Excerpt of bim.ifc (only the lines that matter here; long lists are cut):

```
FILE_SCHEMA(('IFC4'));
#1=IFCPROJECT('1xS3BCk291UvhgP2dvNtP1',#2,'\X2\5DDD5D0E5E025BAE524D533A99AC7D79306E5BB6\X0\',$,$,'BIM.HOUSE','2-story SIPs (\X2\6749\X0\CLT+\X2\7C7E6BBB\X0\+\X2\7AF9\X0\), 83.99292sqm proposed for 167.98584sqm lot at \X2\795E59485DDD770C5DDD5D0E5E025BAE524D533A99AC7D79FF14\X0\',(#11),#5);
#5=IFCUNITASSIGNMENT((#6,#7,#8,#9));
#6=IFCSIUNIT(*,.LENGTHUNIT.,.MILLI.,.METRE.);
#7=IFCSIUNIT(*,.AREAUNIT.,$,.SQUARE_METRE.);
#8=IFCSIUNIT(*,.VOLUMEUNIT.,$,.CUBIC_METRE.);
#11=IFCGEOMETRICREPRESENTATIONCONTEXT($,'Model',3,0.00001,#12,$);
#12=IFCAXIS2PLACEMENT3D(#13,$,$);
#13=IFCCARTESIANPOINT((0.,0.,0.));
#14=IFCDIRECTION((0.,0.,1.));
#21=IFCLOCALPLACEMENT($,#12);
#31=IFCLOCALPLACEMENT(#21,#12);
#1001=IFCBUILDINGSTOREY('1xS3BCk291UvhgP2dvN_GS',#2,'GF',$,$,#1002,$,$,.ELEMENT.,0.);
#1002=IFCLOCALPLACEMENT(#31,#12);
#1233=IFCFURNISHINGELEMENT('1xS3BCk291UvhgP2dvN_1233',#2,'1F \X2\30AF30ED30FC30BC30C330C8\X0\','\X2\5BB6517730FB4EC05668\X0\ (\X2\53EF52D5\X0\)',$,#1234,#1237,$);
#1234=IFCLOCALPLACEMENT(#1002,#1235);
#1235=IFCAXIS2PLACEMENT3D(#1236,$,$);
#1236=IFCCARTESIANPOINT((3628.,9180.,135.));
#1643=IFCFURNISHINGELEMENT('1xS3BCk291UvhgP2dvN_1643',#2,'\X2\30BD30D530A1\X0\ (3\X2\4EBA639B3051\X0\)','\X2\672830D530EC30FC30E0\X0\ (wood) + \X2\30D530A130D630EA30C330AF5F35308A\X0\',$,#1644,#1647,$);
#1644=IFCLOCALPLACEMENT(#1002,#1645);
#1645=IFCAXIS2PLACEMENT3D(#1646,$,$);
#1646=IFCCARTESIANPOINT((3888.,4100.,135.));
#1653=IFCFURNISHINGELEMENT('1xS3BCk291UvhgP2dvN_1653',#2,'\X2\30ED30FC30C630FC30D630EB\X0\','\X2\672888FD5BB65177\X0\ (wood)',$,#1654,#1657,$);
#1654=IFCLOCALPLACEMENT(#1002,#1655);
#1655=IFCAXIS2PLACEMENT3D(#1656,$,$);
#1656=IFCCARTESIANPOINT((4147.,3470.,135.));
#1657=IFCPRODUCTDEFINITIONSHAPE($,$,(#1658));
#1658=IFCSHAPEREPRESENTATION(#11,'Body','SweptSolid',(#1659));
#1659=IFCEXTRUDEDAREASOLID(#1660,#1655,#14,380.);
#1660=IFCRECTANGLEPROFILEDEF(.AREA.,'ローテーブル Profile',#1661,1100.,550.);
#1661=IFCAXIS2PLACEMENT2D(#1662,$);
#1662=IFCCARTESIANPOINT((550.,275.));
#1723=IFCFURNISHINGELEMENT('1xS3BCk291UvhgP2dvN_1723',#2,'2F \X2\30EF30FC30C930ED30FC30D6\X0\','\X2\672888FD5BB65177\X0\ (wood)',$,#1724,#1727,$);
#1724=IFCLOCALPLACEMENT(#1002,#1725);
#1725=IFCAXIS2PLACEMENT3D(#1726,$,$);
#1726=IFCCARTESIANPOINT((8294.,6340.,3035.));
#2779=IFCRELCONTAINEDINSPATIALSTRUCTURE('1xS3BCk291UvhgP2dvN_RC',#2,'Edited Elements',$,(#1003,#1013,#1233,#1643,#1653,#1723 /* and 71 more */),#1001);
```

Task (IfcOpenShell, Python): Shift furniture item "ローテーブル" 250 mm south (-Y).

```python
import ifcopenshell
import ifcopenshell.api.geometry
import ifcopenshell.util.placement
import ifcopenshell.util.unit

model = ifcopenshell.open("bim.ifc")
unit_scale = ifcopenshell.util.unit.calculate_unit_scale(model)

item = model.by_guid("1xS3BCk291UvhgP2dvN_1653")
matrix = ifcopenshell.util.placement.get_local_placement(item.ObjectPlacement)
matrix[1, 3] -= 0.25 / unit_scale
ifcopenshell.api.geometry.edit_object_placement(model, product=item, matrix=matrix, is_si=False)

print(ifcopenshell.util.placement.get_local_placement(item.ObjectPlacement).round(3) + 0.0)

model.write("bim_edited.ifc")
```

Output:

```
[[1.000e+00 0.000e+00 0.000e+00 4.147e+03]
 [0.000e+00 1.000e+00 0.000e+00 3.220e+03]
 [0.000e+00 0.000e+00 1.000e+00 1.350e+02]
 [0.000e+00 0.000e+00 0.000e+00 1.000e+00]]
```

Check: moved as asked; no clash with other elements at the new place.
